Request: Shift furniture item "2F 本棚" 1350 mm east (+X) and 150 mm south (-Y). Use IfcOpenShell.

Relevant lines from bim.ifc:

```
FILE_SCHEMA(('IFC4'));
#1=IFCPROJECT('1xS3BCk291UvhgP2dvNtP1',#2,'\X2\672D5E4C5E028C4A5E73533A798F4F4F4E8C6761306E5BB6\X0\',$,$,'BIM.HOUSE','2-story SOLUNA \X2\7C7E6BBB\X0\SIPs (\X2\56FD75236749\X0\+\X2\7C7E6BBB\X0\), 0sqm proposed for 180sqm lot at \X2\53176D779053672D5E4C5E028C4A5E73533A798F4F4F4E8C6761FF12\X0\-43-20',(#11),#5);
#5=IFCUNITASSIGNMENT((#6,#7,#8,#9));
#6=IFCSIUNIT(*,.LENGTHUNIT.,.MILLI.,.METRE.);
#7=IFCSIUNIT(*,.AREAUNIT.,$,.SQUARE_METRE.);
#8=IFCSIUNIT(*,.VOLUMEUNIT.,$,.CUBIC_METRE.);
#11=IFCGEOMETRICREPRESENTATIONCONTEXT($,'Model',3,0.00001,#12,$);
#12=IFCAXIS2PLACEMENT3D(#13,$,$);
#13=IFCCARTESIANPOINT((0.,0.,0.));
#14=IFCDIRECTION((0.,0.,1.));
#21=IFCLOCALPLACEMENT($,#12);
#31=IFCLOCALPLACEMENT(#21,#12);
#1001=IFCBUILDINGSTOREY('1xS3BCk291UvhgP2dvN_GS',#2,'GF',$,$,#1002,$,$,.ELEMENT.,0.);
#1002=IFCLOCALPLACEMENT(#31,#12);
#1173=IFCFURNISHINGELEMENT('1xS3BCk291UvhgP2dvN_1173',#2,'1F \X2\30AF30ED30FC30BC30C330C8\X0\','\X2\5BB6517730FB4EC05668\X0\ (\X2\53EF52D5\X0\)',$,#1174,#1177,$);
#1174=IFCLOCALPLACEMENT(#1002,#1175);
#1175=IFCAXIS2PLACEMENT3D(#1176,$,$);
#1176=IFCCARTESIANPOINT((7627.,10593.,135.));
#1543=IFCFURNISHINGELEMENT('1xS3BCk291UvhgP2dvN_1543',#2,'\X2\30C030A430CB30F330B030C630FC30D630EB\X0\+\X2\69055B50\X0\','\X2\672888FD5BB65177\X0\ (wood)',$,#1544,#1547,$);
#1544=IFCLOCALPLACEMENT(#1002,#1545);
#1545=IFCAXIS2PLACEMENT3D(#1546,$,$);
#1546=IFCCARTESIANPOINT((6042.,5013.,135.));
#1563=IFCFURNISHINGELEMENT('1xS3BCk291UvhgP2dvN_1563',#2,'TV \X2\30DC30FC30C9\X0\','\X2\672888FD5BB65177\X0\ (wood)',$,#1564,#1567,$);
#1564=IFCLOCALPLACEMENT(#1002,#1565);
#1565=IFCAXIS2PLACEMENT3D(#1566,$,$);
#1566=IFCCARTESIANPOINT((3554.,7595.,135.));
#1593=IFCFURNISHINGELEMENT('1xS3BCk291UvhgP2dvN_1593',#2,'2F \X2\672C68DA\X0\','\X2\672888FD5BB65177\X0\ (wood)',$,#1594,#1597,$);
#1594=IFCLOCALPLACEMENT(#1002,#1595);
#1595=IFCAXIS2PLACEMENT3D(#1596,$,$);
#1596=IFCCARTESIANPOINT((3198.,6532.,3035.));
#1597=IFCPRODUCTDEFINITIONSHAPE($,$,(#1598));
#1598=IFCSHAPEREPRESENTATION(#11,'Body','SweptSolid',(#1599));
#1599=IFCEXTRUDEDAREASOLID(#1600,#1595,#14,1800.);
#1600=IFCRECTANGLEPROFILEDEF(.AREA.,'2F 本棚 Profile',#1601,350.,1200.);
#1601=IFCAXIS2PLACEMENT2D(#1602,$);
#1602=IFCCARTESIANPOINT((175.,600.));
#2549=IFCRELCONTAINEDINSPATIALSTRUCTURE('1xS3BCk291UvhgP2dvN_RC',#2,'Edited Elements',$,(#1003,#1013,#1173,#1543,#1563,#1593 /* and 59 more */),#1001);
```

```python
import ifcopenshell
import ifcopenshell.api.geometry
import ifcopenshell.util.placement
import ifcopenshell.util.unit

model = ifcopenshell.open("bim.ifc")
unit_scale = ifcopenshell.util.unit.calculate_unit_scale(model)

item = model.by_guid("1xS3BCk291UvhgP2dvN_1593")
matrix = ifcopenshell.util.placement.get_local_placement(item.ObjectPlacement)
matrix[0, 3] += 1.35 / unit_scale
matrix[1, 3] -= 0.15 / unit_scale
ifcopenshell.api.geometry.edit_object_placement(model, product=item, matrix=matrix, is_si=False)

print(ifcopenshell.util.placement.get_local_placement(item.ObjectPlacement).round(3) + 0.0)

model.write("bim_v2.ifc")
```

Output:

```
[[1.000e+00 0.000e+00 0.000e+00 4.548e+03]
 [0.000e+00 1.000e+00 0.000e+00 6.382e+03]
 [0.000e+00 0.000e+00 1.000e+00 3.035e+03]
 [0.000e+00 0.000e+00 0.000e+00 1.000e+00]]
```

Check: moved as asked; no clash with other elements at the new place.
